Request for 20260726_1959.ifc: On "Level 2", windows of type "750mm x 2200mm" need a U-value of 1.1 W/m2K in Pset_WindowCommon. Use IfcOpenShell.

First a look at what the model holds.

```python
import ifcopenshell
import ifcopenshell.util.element

model = ifcopenshell.open("20260726_1959.ifc")
print(model.schema)
storey = next(s for s in model.by_type("IfcBuildingStorey") if s.Name == "Level 2")
windows = [e for e in ifcopenshell.util.element.get_decomposition(storey) if e.is_a("IfcWindow")]
seen = {}
for e in windows:
    element_type = ifcopenshell.util.element.get_type(e)
    key = (element_type.Name if element_type != e and element_type else None, ifcopenshell.util.element.get_pset(e, "Pset_WindowCommon", "ThermalTransmittance"))
    seen[key] = seen.get(key, 0) + 1
for (name, value), count in sorted(seen.items(), key=str):
    print(count, "x", name, "|", value)
```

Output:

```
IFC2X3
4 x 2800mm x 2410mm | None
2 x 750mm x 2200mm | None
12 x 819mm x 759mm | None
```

```python
import ifcopenshell
import ifcopenshell.api.pset
import ifcopenshell.util.element

model = ifcopenshell.open("20260726_1959.ifc")

storey = next(s for s in model.by_type("IfcBuildingStorey") if s.Name == "Level 2")
windows = [e for e in ifcopenshell.util.element.get_decomposition(storey) if e.is_a("IfcWindow")]

count = 0
for e in windows:
    element_type = ifcopenshell.util.element.get_type(e)
    if element_type in (None, e) or element_type.Name != "750mm x 2200mm":
        continue
    # add_pset returns the element's existing set when there is one.
    pset = ifcopenshell.api.pset.add_pset(model, product=e, name="Pset_WindowCommon")
    ifcopenshell.api.pset.edit_pset(model, pset=pset, properties={"ThermalTransmittance": 1.1})
    count += 1

print(count, "windows updated")

model.write("20260726_1959_v2.ifc")
```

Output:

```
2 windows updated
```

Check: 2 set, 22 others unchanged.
